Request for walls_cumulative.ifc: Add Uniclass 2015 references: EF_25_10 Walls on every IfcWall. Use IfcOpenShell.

First a look at what the model holds.

```python
import ifcopenshell

model = ifcopenshell.open("walls_cumulative.ifc")
print(model.schema)
print("classifications:", [c.Name for c in model.by_type("IfcClassification")])
for ifc_class in ("IfcDoor", "IfcRoof", "IfcStair", "IfcWall", "IfcWindow"):
    print(ifc_class, len(model.by_type(ifc_class)))
```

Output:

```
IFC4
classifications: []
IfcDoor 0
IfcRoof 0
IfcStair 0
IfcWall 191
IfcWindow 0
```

```python
import ifcopenshell
import ifcopenshell.api.classification

model = ifcopenshell.open("walls_cumulative.ifc")

system = ifcopenshell.api.classification.add_classification(model, classification="Uniclass 2015")

codes = {
    "IfcWall": ("EF_25_10", "Walls"),
}
for ifc_class, (code, name) in codes.items():
    products = model.by_type(ifc_class)
    ifcopenshell.api.classification.add_reference(
        model, products=products, classification=system, identification=code, name=name
    )
    print(code, len(products))

model.write("walls_cumulative_rev.ifc")
```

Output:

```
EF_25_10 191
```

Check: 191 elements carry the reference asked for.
